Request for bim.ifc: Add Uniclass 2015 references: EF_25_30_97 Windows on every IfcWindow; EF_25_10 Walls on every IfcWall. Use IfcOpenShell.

First a look at what the model holds.

```python
import ifcopenshell

model = ifcopenshell.open("bim.ifc")
print(model.schema)
print("classifications:", [c.Name for c in model.by_type("IfcClassification")])
for ifc_class in ("IfcDoor", "IfcRoof", "IfcStair", "IfcWall", "IfcWindow"):
    print(ifc_class, len(model.by_type(ifc_class)))
```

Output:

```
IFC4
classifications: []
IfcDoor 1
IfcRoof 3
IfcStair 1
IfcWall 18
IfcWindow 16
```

```python
import ifcopenshell
import ifcopenshell.api.classification

model = ifcopenshell.open("bim.ifc")

system = ifcopenshell.api.classification.add_classification(model, classification="Uniclass 2015")

codes = {
    "IfcWindow": ("EF_25_30_97", "Windows"),
    "IfcWall": ("EF_25_10", "Walls"),
}
for ifc_class, (code, name) in codes.items():
    products = model.by_type(ifc_class)
    ifcopenshell.api.classification.add_reference(
        model, products=products, classification=system, identification=code, name=name
    )
    print(code, len(products))

model.write("bim-out.ifc")
```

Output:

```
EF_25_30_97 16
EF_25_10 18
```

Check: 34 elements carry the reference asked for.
